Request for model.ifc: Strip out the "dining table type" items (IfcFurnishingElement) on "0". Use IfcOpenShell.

First a look at what the model holds.

```python
import ifcopenshell
import ifcopenshell.util.element

model = ifcopenshell.open("model.ifc")
print(model.schema)
storey = next(s for s in model.by_type("IfcBuildingStorey") if s.Name == "0")
furniture = [e for e in ifcopenshell.util.element.get_decomposition(storey) if e.is_a("IfcFurnishingElement")]
seen = {}
for e in furniture:
    element_type = ifcopenshell.util.element.get_type(e)
    name = element_type.Name if element_type not in (None, e) else None
    seen[name] = seen.get(name, 0) + 1
for name, count in sorted(seen.items(), key=str):
    print(count, "x", name)
```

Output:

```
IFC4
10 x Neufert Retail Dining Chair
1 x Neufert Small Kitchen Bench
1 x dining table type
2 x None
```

```python
import ifcopenshell
import ifcopenshell.api.root
import ifcopenshell.util.element

model = ifcopenshell.open("model.ifc")

storey = next(s for s in model.by_type("IfcBuildingStorey") if s.Name == "0")
furniture = [e for e in ifcopenshell.util.element.get_decomposition(storey) if e.is_a("IfcFurnishingElement")]
targets = [e for e in furniture if (t := ifcopenshell.util.element.get_type(e)) not in (None, e) and t.Name == "dining table type"]

for e in targets:
    ifcopenshell.api.root.remove_product(model, product=e)
print(len(targets), "removed")

model.write("model-out.ifc")
```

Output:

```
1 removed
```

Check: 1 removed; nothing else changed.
